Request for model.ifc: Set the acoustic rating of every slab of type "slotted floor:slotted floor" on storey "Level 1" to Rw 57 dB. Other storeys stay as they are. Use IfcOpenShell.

First a look at what the model holds.

```python
import ifcopenshell
import ifcopenshell.util.element

model = ifcopenshell.open("model.ifc")
print(model.schema)
storey = next(s for s in model.by_type("IfcBuildingStorey") if s.Name == "Level 1")
slabs = [e for e in ifcopenshell.util.element.get_decomposition(storey) if e.is_a("IfcSlab")]
seen = {}
for e in slabs:
    element_type = ifcopenshell.util.element.get_type(e)
    key = (element_type.Name if element_type != e and element_type else None, ifcopenshell.util.element.get_pset(e, "Pset_SlabCommon", "AcousticRating"))
    seen[key] = seen.get(key, 0) + 1
for (name, value), count in sorted(seen.items(), key=str):
    print(count, "x", name, "|", value)
```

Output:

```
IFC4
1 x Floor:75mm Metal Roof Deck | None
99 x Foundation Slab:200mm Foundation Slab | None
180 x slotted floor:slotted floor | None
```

```python
import ifcopenshell
import ifcopenshell.api.pset
import ifcopenshell.util.element

model = ifcopenshell.open("model.ifc")

storey = next(s for s in model.by_type("IfcBuildingStorey") if s.Name == "Level 1")
slabs = [e for e in ifcopenshell.util.element.get_decomposition(storey) if e.is_a("IfcSlab")]

count = 0
for e in slabs:
    element_type = ifcopenshell.util.element.get_type(e)
    if element_type in (None, e) or element_type.Name != "slotted floor:slotted floor":
        continue
    # add_pset returns the element's existing set when there is one.
    pset = ifcopenshell.api.pset.add_pset(model, product=e, name="Pset_SlabCommon")
    ifcopenshell.api.pset.edit_pset(model, pset=pset, properties={"AcousticRating": "Rw 57 dB"})
    count += 1

print(count, "slabs updated")

model.write("model_rev.ifc")
```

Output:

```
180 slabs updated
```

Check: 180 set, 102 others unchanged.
